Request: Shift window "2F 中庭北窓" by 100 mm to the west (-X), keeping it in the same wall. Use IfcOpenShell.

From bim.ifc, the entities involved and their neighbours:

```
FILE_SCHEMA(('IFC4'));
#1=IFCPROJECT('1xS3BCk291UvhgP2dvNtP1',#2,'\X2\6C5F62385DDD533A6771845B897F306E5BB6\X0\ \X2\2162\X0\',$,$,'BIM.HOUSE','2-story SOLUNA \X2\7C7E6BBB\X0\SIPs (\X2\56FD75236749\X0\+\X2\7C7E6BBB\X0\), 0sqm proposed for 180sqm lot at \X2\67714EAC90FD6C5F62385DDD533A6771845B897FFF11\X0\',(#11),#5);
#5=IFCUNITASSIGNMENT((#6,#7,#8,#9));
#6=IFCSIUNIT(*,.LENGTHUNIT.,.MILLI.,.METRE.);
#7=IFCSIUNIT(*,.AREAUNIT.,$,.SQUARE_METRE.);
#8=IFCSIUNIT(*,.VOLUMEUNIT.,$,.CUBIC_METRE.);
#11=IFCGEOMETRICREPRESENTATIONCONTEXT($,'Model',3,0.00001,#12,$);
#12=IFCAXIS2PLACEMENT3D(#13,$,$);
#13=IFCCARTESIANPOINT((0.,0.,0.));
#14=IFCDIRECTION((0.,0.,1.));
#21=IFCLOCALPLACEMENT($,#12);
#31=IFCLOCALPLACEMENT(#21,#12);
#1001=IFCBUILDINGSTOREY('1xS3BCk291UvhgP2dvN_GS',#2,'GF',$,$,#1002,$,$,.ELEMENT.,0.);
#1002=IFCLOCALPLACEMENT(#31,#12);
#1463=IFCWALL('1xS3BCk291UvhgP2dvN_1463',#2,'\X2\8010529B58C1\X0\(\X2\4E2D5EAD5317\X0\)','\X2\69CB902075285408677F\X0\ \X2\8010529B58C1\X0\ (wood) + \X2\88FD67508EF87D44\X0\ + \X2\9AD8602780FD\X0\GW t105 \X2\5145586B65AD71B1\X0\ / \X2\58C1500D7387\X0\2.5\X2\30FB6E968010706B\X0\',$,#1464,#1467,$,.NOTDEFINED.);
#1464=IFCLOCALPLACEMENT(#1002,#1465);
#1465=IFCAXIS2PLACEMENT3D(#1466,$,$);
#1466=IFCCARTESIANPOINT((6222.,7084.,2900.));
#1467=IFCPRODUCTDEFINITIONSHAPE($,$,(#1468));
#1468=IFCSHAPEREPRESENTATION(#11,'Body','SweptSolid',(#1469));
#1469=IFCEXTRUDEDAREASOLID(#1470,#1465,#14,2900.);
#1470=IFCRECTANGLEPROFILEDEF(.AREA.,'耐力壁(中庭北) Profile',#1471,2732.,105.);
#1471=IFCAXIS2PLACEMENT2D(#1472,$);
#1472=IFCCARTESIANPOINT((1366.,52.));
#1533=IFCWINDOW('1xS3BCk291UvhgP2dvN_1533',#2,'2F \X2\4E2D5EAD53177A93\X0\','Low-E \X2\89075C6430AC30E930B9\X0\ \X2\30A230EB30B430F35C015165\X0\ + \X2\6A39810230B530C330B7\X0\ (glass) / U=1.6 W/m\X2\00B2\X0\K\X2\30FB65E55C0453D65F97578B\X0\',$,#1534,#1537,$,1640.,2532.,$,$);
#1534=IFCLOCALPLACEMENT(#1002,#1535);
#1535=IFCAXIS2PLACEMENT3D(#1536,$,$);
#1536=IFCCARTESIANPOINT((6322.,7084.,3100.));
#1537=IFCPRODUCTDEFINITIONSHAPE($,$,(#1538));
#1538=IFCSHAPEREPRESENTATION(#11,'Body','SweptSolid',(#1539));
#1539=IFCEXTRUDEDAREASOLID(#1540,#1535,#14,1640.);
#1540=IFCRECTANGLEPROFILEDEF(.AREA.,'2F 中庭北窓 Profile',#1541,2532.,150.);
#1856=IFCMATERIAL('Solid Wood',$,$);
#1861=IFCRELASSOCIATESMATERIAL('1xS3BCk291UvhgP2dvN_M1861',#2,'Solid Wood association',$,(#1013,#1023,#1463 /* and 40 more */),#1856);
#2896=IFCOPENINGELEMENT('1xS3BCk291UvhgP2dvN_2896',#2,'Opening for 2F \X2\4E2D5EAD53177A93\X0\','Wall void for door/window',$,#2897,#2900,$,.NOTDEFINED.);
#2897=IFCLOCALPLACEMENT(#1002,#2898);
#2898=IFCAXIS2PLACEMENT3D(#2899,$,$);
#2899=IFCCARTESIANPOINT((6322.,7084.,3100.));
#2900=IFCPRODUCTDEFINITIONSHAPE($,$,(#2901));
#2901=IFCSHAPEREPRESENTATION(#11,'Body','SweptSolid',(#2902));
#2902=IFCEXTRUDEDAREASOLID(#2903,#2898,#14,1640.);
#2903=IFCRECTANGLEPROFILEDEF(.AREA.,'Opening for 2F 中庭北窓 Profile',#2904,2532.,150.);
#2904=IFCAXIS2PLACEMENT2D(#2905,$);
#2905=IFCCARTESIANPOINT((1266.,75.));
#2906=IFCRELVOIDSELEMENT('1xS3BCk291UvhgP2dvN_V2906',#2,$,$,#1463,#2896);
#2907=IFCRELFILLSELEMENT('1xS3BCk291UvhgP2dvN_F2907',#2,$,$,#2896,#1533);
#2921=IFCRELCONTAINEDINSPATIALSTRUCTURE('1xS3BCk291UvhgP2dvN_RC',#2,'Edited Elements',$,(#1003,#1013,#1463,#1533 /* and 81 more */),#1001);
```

```python
import ifcopenshell
import ifcopenshell.api.geometry
import ifcopenshell.util.placement
import ifcopenshell.util.unit

model = ifcopenshell.open("bim.ifc")
unit_scale = ifcopenshell.util.unit.calculate_unit_scale(model)

window = model.by_guid("1xS3BCk291UvhgP2dvN_1533")
opening = window.FillsVoids[0].RelatingOpeningElement
wall = opening.VoidsElements[0].RelatingBuildingElement

wall_matrix = ifcopenshell.util.placement.get_local_placement(wall.ObjectPlacement)
shift = wall_matrix[:3, 0] * -0.1 / unit_scale
before = ifcopenshell.util.placement.get_local_placement(window.ObjectPlacement)[:3, 3].copy()

# The window is not placed relative to its opening, so move both.
for product in (opening, window):
    matrix = ifcopenshell.util.placement.get_local_placement(product.ObjectPlacement)
    matrix[:3, 3] += shift
    ifcopenshell.api.geometry.edit_object_placement(model, product=product, matrix=matrix, is_si=False)

after = ifcopenshell.util.placement.get_local_placement(window.ObjectPlacement)[:3, 3]
print("window moved by", (after - before).round(3) + 0.0)

model.write("bim_updated.ifc")
```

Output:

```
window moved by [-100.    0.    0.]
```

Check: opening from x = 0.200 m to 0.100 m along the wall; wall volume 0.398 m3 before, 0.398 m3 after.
